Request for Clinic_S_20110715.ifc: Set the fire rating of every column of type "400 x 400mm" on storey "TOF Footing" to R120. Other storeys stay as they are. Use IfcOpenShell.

First a look at what the model holds.

```python
import ifcopenshell
import ifcopenshell.util.element

model = ifcopenshell.open("Clinic_S_20110715.ifc")
print(model.schema)
storey = next(s for s in model.by_type("IfcBuildingStorey") if s.Name == "TOF Footing")
columns = [e for e in ifcopenshell.util.element.get_decomposition(storey) if e.is_a("IfcColumn")]
seen = {}
for e in columns:
    element_type = ifcopenshell.util.element.get_type(e)
    key = (element_type.Name if element_type != e and element_type else None, ifcopenshell.util.element.get_pset(e, "Pset_ColumnCommon", "FireRating"))
    seen[key] = seen.get(key, 0) + 1
for (name, value), count in sorted(seen.items(), key=str):
    print(count, "x", name, "|", value)
```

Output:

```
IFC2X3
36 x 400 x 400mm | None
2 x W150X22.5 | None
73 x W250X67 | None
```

```python
import ifcopenshell
import ifcopenshell.api.pset
import ifcopenshell.util.element

model = ifcopenshell.open("Clinic_S_20110715.ifc")

storey = next(s for s in model.by_type("IfcBuildingStorey") if s.Name == "TOF Footing")
columns = [e for e in ifcopenshell.util.element.get_decomposition(storey) if e.is_a("IfcColumn")]

count = 0
for e in columns:
    element_type = ifcopenshell.util.element.get_type(e)
    if element_type in (None, e) or element_type.Name != "400 x 400mm":
        continue
    # add_pset returns the element's existing set when there is one.
    pset = ifcopenshell.api.pset.add_pset(model, product=e, name="Pset_ColumnCommon")
    ifcopenshell.api.pset.edit_pset(model, pset=pset, properties={"FireRating": "R120"})
    count += 1

print(count, "columns updated")

model.write("Clinic_S_20110715_rev.ifc")
```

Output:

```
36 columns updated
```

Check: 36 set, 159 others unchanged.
